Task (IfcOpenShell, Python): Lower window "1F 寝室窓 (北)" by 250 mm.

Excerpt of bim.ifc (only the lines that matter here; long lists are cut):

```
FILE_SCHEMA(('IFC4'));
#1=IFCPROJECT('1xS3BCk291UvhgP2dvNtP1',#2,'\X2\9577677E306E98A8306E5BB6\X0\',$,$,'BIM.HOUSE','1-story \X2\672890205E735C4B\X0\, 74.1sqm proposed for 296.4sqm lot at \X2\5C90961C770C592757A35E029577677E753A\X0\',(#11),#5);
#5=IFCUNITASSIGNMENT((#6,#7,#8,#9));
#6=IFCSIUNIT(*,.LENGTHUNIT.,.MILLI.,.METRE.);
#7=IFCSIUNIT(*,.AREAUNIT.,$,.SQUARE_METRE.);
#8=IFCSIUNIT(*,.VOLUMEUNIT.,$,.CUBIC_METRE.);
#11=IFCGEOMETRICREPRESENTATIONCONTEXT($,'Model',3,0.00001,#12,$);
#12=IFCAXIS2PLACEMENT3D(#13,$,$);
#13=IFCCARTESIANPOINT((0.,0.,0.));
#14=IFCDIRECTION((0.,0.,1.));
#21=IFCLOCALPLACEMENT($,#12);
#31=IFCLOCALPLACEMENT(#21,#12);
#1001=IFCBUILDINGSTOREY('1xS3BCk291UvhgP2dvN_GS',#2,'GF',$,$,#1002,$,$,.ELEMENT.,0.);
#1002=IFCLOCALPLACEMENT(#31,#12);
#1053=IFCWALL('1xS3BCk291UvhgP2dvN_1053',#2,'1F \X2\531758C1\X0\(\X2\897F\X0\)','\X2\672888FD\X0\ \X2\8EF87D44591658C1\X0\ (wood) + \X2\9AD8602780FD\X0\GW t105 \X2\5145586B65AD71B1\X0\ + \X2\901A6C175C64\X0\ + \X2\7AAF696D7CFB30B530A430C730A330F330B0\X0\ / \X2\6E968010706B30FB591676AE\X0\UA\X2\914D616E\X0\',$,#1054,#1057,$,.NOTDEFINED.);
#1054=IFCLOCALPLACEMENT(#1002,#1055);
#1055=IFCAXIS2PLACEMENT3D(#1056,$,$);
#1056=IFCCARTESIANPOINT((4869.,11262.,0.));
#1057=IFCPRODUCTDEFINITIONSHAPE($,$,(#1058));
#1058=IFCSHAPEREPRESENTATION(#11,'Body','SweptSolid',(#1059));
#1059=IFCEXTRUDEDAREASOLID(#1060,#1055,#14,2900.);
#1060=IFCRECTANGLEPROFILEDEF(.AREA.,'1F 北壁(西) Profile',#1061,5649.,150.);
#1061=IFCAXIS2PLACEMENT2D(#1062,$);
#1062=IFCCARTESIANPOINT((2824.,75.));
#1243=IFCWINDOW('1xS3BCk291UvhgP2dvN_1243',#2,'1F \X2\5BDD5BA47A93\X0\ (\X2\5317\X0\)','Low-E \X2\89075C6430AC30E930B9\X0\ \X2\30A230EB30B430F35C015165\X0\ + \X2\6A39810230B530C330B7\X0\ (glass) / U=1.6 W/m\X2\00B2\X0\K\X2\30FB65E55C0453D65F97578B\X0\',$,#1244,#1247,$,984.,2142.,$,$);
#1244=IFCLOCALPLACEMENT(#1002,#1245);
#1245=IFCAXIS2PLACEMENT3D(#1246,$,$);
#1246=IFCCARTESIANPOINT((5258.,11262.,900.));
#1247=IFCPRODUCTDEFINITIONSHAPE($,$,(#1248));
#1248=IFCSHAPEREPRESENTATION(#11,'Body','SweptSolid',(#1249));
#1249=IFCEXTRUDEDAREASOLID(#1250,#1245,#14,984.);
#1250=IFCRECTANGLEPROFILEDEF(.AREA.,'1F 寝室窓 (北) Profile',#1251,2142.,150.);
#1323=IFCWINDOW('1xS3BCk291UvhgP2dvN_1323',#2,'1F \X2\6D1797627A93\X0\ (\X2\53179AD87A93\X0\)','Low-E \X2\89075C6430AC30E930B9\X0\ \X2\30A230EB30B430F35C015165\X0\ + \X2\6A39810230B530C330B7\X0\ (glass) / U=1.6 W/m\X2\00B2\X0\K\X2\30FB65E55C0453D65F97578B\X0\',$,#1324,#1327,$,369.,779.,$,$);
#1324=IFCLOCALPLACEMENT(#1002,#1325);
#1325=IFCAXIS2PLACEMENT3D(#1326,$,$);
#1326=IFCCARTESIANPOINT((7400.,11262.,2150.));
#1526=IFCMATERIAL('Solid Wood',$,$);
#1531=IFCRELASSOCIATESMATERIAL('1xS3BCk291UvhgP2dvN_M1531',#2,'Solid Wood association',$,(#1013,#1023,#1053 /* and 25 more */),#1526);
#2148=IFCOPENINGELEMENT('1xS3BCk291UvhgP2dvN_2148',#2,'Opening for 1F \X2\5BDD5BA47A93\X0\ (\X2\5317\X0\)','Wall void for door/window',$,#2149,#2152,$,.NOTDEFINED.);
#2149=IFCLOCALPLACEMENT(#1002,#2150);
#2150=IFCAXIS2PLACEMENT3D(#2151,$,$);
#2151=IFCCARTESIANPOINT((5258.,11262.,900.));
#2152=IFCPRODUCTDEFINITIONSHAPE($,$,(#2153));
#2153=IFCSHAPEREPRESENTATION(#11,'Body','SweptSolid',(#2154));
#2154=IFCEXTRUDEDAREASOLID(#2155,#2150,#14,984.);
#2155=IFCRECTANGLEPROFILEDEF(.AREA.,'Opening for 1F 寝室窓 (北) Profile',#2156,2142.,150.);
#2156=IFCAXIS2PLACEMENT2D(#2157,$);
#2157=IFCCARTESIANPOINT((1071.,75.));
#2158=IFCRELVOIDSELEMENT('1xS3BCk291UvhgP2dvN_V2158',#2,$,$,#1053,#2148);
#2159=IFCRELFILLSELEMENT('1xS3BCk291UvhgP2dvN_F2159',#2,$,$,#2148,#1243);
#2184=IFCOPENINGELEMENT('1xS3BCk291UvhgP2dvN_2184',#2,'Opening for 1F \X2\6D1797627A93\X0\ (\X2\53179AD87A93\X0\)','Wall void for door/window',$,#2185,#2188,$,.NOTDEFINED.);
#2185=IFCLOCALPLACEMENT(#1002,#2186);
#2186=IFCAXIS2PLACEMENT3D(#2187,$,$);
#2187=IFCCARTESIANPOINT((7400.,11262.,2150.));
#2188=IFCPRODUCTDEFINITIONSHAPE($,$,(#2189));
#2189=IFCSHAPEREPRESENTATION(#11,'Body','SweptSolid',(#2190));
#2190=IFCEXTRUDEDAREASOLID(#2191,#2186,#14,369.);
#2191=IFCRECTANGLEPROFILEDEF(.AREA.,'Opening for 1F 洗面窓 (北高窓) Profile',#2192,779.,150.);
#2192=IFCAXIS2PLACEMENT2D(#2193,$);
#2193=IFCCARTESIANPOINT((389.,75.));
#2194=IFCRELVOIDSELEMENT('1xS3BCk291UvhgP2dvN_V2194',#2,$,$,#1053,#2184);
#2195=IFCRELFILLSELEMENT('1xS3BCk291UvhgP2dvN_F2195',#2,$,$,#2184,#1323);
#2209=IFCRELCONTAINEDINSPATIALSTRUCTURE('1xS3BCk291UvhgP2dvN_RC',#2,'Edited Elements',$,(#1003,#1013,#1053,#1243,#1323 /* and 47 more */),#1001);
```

```python
import numpy as np
import ifcopenshell
import ifcopenshell.api.geometry
import ifcopenshell.util.placement
import ifcopenshell.util.unit

model = ifcopenshell.open("bim.ifc")
unit_scale = ifcopenshell.util.unit.calculate_unit_scale(model)

window = model.by_id(1243)
opening = window.FillsVoids[0].RelatingOpeningElement
dz = -0.25 / unit_scale

shift = np.array([0.0, 0.0, dz])
# The window is not placed relative to its opening, so move both.
for product in (opening, window):
    matrix = ifcopenshell.util.placement.get_local_placement(product.ObjectPlacement)
    matrix[:3, 3] += shift
    ifcopenshell.api.geometry.edit_object_placement(model, product=product, matrix=matrix, is_si=False)

print(f"moved by {dz * unit_scale:+.3f} m")

model.write("bim_updated.ifc")
```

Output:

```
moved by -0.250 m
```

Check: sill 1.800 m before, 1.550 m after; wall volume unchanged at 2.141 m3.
